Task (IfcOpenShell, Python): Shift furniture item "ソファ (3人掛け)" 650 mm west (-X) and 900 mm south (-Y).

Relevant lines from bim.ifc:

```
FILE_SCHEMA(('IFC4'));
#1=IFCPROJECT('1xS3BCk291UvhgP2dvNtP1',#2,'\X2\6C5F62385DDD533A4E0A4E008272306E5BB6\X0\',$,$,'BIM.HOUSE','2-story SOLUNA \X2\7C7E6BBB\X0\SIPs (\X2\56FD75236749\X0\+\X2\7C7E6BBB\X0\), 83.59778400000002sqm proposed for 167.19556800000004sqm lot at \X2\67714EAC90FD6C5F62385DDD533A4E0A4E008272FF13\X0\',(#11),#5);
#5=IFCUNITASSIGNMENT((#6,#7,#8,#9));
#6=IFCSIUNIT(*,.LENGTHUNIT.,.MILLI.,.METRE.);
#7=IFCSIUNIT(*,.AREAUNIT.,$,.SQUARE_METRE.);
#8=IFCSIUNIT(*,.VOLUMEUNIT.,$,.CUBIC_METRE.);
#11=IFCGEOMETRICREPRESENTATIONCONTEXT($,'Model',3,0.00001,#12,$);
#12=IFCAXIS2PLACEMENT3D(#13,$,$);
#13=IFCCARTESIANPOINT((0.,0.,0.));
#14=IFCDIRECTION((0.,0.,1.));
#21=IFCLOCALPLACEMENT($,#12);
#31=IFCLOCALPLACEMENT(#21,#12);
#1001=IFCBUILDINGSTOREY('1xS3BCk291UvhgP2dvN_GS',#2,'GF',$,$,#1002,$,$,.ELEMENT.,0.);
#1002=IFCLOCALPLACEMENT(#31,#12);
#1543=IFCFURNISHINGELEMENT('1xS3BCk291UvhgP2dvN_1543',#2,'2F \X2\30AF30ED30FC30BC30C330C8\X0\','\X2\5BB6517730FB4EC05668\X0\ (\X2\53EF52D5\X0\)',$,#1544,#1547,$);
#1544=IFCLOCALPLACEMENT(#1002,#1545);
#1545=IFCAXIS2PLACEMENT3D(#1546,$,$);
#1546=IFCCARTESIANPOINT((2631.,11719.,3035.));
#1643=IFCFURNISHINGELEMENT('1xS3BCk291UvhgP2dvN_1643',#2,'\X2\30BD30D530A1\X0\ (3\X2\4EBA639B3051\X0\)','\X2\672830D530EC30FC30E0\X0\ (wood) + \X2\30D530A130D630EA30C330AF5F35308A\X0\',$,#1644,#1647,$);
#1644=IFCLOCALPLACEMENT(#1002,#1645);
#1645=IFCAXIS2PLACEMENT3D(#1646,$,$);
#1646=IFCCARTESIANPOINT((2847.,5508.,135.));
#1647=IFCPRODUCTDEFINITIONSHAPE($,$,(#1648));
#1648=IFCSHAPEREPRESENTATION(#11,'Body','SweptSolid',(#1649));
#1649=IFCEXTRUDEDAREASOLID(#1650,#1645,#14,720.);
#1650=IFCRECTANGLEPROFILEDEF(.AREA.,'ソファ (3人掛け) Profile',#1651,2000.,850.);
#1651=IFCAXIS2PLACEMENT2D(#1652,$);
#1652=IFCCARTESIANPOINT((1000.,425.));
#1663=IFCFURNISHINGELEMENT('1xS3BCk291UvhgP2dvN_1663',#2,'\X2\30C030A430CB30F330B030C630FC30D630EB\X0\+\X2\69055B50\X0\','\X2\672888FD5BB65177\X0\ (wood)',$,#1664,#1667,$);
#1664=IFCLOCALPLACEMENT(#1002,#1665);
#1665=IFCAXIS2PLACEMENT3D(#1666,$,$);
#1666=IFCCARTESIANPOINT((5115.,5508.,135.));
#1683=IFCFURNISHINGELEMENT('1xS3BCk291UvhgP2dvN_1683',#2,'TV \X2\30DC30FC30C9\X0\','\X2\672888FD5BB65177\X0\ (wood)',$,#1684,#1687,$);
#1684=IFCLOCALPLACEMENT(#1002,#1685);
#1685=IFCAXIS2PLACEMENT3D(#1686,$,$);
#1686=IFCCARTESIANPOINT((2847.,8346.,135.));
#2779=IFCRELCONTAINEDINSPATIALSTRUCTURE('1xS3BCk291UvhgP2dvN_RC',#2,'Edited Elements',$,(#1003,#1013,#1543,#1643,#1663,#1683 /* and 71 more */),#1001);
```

```python
import ifcopenshell
import ifcopenshell.api.geometry
import ifcopenshell.util.placement
import ifcopenshell.util.unit

model = ifcopenshell.open("bim.ifc")
unit_scale = ifcopenshell.util.unit.calculate_unit_scale(model)

item = model.by_guid("1xS3BCk291UvhgP2dvN_1643")
matrix = ifcopenshell.util.placement.get_local_placement(item.ObjectPlacement)
matrix[0, 3] -= 0.65 / unit_scale
matrix[1, 3] -= 0.9 / unit_scale
ifcopenshell.api.geometry.edit_object_placement(model, product=item, matrix=matrix, is_si=False)

print(ifcopenshell.util.placement.get_local_placement(item.ObjectPlacement).round(3) + 0.0)

model.write("bim_edited.ifc")
```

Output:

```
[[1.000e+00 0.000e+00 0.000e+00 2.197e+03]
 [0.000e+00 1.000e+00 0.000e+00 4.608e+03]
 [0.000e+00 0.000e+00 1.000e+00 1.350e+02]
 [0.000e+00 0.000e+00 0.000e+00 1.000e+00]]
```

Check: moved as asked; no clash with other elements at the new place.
